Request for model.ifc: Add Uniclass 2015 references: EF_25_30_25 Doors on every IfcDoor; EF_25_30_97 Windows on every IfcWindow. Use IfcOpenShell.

First a look at what the model holds.

```python
import ifcopenshell

model = ifcopenshell.open("model.ifc")
print(model.schema)
print("classifications:", [c.Name for c in model.by_type("IfcClassification")])
for ifc_class in ("IfcDoor", "IfcRoof", "IfcStair", "IfcWall", "IfcWindow"):
    print(ifc_class, len(model.by_type(ifc_class)))
```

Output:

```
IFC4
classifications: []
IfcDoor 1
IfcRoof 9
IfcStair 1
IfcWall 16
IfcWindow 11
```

```python
import ifcopenshell
import ifcopenshell.api.classification

model = ifcopenshell.open("model.ifc")

system = ifcopenshell.api.classification.add_classification(model, classification="Uniclass 2015")

codes = {
    "IfcDoor": ("EF_25_30_25", "Doors"),
    "IfcWindow": ("EF_25_30_97", "Windows"),
}
for ifc_class, (code, name) in codes.items():
    products = model.by_type(ifc_class)
    ifcopenshell.api.classification.add_reference(
        model, products=products, classification=system, identification=code, name=name
    )
    print(code, len(products))

model.write("model_rev.ifc")
```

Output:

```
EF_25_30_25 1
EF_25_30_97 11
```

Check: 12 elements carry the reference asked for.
